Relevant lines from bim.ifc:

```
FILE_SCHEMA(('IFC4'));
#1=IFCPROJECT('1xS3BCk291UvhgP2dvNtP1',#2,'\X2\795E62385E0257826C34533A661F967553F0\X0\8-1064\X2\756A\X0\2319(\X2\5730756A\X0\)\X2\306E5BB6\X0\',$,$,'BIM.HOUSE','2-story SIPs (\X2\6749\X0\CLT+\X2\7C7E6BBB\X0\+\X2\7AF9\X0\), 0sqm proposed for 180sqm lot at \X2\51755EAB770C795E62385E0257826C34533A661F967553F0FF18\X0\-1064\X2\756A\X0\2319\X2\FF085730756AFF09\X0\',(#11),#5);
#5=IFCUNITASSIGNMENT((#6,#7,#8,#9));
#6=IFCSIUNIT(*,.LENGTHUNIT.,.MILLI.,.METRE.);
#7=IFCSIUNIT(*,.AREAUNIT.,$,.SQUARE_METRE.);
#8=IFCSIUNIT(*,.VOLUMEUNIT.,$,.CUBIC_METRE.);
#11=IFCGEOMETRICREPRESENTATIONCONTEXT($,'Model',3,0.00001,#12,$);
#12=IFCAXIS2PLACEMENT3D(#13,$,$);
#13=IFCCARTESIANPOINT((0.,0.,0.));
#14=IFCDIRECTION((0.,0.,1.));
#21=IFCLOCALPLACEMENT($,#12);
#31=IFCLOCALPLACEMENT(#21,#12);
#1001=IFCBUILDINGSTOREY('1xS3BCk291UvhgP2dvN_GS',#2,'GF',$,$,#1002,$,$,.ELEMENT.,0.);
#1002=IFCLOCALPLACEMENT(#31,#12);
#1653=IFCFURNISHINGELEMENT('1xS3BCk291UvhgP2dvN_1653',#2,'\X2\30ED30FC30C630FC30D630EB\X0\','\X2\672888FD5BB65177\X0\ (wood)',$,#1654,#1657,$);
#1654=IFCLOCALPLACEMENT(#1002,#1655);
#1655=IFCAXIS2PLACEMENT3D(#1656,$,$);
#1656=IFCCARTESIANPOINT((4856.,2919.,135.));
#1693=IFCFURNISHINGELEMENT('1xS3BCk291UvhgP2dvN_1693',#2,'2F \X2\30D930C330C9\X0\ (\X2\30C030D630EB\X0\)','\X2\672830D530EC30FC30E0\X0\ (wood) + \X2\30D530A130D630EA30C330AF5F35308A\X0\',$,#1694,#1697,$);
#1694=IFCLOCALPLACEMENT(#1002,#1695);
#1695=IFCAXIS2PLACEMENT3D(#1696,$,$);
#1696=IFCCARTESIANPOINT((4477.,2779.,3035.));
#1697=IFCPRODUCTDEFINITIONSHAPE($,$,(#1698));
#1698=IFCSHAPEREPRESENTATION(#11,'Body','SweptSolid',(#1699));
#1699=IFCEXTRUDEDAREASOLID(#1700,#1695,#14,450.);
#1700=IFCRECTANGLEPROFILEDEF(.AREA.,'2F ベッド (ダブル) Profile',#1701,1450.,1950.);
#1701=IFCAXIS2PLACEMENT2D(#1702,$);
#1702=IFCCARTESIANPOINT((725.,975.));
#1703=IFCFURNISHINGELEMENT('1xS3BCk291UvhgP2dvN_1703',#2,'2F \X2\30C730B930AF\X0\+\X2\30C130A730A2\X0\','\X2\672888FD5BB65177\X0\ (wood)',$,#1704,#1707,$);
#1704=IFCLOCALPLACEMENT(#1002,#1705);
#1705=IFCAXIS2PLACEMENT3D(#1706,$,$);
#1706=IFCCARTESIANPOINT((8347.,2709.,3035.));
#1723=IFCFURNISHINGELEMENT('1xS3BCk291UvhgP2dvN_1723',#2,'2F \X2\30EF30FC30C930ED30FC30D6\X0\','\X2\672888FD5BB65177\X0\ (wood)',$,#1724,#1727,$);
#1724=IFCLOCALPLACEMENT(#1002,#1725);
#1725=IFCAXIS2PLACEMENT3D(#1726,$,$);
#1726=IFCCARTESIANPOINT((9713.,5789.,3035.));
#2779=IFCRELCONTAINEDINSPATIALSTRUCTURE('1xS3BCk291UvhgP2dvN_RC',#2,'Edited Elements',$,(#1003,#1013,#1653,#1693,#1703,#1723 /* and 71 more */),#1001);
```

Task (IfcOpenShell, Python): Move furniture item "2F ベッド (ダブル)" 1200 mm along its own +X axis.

```python
import ifcopenshell
import ifcopenshell.api.geometry
import ifcopenshell.util.placement

model = ifcopenshell.open("bim.ifc")

item = model.by_guid("1xS3BCk291UvhgP2dvN_1693")
matrix = ifcopenshell.util.placement.get_local_placement(item.ObjectPlacement)
matrix[:3, 3] += matrix[:3, 0] * 1200.0
ifcopenshell.api.geometry.edit_object_placement(model, product=item, matrix=matrix, is_si=False)

print(ifcopenshell.util.placement.get_local_placement(item.ObjectPlacement).round(3) + 0.0)

model.write("bim-out.ifc")
```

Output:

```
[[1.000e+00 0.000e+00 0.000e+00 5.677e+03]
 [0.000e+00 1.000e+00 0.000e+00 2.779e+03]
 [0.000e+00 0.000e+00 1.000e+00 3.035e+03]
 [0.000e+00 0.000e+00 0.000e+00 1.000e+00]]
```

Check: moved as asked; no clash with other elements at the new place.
